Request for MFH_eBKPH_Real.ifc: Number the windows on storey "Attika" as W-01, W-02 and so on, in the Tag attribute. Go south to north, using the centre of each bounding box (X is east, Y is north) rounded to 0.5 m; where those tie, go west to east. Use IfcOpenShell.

First a look at what the model holds.

```python
import ifcopenshell
import ifcopenshell.util.element
import ifcopenshell.util.placement

model = ifcopenshell.open("MFH_eBKPH_Real.ifc")
print(model.schema)
storey = next(s for s in model.by_type("IfcBuildingStorey") if s.Name == "Attika")
windows = [e for e in ifcopenshell.util.element.get_decomposition(storey) if e.is_a("IfcWindow")]
for e in sorted(windows, key=lambda e: e.id()):
    origin = ifcopenshell.util.placement.get_local_placement(e.ObjectPlacement)[:3, 3]
    print(e.id(), e.Tag, e.Name, origin.round(2) + 0.0, sep=" | ")
```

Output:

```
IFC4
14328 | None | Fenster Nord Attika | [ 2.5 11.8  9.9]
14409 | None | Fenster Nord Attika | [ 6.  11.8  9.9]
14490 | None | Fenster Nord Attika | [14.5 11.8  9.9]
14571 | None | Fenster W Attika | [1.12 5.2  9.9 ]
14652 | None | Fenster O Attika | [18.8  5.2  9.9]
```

```python
import ifcopenshell
import ifcopenshell.geom
import ifcopenshell.util.element
import ifcopenshell.util.shape

model = ifcopenshell.open("MFH_eBKPH_Real.ifc")
settings = ifcopenshell.geom.settings()
settings.set("use-world-coords", True)


def centre(element):
    shape = ifcopenshell.geom.create_shape(settings, element)
    return ifcopenshell.util.shape.get_bbox_centroid(shape.geometry)


storey = next(s for s in model.by_type("IfcBuildingStorey") if s.Name == "Attika")
windows = [e for e in ifcopenshell.util.element.get_decomposition(storey) if e.is_a("IfcWindow")]

# Insertion points can sit at a corner or the storey origin, so sort by the geometry (in metres).
centres = {e: centre(e) for e in windows}
windows.sort(key=lambda e: (round(centres[e][1] / 0.5), centres[e][0]))

for i, e in enumerate(windows, start=1):
    number = f"W-{i:02d}"
    e.Tag = number
    print(e.id(), number)

model.write("MFH_eBKPH_Real_v2.ifc")
```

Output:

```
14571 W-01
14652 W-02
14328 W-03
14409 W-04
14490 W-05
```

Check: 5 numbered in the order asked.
